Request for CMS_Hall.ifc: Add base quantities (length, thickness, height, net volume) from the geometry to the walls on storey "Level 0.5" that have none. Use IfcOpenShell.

First a look at what the model holds.

```python
import ifcopenshell
import ifcopenshell.util.element
import ifcopenshell.util.unit

model = ifcopenshell.open("CMS_Hall.ifc")
print(model.schema)
for unit_type in ("LENGTHUNIT", "AREAUNIT", "VOLUMEUNIT"):
    print(unit_type, ifcopenshell.util.unit.calculate_unit_scale(model, unit_type))
storey = next(s for s in model.by_type("IfcBuildingStorey") if s.Name == "Level 0.5")
walls = [e for e in ifcopenshell.util.element.get_decomposition(storey) if e.is_a("IfcWall")]
for e in sorted(walls, key=lambda e: e.id()):
    print(e.id(), e.is_a(), e.Name, list(ifcopenshell.util.element.get_psets(e, qtos_only=True)), sep=" | ")
```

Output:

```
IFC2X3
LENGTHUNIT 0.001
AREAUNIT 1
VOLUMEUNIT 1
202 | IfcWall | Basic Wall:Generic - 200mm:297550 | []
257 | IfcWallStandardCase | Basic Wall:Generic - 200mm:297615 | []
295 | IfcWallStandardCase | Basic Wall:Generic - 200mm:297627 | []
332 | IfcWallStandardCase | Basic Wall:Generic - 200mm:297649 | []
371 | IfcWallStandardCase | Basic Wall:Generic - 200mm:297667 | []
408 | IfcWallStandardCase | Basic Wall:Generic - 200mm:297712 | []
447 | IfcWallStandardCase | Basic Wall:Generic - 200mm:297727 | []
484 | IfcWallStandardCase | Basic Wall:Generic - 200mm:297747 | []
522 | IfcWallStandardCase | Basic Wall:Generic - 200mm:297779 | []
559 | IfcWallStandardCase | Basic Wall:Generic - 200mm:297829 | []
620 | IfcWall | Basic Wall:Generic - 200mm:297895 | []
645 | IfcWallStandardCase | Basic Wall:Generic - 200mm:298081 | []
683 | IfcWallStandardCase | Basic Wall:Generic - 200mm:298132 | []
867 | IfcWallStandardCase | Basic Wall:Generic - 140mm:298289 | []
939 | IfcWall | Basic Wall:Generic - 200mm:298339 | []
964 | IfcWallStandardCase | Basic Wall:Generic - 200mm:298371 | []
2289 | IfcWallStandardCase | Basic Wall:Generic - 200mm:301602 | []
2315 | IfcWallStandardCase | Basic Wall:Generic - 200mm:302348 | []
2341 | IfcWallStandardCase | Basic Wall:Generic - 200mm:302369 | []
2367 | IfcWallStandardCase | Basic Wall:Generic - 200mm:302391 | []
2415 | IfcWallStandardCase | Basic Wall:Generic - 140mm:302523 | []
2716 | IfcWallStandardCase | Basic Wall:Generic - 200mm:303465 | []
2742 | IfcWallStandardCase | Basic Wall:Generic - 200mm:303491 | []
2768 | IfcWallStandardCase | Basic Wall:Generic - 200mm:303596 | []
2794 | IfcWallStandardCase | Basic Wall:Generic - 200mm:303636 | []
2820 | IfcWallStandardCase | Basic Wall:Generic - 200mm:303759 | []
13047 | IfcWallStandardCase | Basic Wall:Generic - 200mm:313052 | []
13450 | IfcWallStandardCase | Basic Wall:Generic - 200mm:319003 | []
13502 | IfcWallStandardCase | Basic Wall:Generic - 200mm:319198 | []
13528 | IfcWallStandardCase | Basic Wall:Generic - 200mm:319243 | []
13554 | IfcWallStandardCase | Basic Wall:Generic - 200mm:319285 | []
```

```python
import ifcopenshell
import ifcopenshell.api.pset
import ifcopenshell.geom
import ifcopenshell.util.element
import ifcopenshell.util.shape
import ifcopenshell.util.unit

model = ifcopenshell.open("CMS_Hall.ifc")
unit_scale = ifcopenshell.util.unit.calculate_unit_scale(model)
volume_scale = ifcopenshell.util.unit.calculate_unit_scale(model, "VOLUMEUNIT")
settings = ifcopenshell.geom.settings()

storey = next(s for s in model.by_type("IfcBuildingStorey") if s.Name == "Level 0.5")
walls = [e for e in ifcopenshell.util.element.get_decomposition(storey) if e.is_a("IfcWall")]

for e in sorted(walls, key=lambda e: e.id()):
    if ifcopenshell.util.element.get_psets(e, qtos_only=True, should_inherit=False):
        continue
    # Geometry comes back in metres, in the element's own axes.
    shape = ifcopenshell.geom.create_shape(settings, e)
    values = {
        "Length": ifcopenshell.util.shape.get_x(shape.geometry) / unit_scale,
        "Width": ifcopenshell.util.shape.get_y(shape.geometry) / unit_scale,
        "Height": ifcopenshell.util.shape.get_z(shape.geometry) / unit_scale,
        "NetVolume": ifcopenshell.util.shape.get_volume(shape.geometry) / volume_scale,
    }
    qto = ifcopenshell.api.pset.add_qto(model, product=e, name="BaseQuantities")
    ifcopenshell.api.pset.edit_qto(model, qto=qto, properties=values)
    print(e.id(), {k: round(v, 3) for k, v in values.items()})

model.write("CMS_Hall-out.ifc")
```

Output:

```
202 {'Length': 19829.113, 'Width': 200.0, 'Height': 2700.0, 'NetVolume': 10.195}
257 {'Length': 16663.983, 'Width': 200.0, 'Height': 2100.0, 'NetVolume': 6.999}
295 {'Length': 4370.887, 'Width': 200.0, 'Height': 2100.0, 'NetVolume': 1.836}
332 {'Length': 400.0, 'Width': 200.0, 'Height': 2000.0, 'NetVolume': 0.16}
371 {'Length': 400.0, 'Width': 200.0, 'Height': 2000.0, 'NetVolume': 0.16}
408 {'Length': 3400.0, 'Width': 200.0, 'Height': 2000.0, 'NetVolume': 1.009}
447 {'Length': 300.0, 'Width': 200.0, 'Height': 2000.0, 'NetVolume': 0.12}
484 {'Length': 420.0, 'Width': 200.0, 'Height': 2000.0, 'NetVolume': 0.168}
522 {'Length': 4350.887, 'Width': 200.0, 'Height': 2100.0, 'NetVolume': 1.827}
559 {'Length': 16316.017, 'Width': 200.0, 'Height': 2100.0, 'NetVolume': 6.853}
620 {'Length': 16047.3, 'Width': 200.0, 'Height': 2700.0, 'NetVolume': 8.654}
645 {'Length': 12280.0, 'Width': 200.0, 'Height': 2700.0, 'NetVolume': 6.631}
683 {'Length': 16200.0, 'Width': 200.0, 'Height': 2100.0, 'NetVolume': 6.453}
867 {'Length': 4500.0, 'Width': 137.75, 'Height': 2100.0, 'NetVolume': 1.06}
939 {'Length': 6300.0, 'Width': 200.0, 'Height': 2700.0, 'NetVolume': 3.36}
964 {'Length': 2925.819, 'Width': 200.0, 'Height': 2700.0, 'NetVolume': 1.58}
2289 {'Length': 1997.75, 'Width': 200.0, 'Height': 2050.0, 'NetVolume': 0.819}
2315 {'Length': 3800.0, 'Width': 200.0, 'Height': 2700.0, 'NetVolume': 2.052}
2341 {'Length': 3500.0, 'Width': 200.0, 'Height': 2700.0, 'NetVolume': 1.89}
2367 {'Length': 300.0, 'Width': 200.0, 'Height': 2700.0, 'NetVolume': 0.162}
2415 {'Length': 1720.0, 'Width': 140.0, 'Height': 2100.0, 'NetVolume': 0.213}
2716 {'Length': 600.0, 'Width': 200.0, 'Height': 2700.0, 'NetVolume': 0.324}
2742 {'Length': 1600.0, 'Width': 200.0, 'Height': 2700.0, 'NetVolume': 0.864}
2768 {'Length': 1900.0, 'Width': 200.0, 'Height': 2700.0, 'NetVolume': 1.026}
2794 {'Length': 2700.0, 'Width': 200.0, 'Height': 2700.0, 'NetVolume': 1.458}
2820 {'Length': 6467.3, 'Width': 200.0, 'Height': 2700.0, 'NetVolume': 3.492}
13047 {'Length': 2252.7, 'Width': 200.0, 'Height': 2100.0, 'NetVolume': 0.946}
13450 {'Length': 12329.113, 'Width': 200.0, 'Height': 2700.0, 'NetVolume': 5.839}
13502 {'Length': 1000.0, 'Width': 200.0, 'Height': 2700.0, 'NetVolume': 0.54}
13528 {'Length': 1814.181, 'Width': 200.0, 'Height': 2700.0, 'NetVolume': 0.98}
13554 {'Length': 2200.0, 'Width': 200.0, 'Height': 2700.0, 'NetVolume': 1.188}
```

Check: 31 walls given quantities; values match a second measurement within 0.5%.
